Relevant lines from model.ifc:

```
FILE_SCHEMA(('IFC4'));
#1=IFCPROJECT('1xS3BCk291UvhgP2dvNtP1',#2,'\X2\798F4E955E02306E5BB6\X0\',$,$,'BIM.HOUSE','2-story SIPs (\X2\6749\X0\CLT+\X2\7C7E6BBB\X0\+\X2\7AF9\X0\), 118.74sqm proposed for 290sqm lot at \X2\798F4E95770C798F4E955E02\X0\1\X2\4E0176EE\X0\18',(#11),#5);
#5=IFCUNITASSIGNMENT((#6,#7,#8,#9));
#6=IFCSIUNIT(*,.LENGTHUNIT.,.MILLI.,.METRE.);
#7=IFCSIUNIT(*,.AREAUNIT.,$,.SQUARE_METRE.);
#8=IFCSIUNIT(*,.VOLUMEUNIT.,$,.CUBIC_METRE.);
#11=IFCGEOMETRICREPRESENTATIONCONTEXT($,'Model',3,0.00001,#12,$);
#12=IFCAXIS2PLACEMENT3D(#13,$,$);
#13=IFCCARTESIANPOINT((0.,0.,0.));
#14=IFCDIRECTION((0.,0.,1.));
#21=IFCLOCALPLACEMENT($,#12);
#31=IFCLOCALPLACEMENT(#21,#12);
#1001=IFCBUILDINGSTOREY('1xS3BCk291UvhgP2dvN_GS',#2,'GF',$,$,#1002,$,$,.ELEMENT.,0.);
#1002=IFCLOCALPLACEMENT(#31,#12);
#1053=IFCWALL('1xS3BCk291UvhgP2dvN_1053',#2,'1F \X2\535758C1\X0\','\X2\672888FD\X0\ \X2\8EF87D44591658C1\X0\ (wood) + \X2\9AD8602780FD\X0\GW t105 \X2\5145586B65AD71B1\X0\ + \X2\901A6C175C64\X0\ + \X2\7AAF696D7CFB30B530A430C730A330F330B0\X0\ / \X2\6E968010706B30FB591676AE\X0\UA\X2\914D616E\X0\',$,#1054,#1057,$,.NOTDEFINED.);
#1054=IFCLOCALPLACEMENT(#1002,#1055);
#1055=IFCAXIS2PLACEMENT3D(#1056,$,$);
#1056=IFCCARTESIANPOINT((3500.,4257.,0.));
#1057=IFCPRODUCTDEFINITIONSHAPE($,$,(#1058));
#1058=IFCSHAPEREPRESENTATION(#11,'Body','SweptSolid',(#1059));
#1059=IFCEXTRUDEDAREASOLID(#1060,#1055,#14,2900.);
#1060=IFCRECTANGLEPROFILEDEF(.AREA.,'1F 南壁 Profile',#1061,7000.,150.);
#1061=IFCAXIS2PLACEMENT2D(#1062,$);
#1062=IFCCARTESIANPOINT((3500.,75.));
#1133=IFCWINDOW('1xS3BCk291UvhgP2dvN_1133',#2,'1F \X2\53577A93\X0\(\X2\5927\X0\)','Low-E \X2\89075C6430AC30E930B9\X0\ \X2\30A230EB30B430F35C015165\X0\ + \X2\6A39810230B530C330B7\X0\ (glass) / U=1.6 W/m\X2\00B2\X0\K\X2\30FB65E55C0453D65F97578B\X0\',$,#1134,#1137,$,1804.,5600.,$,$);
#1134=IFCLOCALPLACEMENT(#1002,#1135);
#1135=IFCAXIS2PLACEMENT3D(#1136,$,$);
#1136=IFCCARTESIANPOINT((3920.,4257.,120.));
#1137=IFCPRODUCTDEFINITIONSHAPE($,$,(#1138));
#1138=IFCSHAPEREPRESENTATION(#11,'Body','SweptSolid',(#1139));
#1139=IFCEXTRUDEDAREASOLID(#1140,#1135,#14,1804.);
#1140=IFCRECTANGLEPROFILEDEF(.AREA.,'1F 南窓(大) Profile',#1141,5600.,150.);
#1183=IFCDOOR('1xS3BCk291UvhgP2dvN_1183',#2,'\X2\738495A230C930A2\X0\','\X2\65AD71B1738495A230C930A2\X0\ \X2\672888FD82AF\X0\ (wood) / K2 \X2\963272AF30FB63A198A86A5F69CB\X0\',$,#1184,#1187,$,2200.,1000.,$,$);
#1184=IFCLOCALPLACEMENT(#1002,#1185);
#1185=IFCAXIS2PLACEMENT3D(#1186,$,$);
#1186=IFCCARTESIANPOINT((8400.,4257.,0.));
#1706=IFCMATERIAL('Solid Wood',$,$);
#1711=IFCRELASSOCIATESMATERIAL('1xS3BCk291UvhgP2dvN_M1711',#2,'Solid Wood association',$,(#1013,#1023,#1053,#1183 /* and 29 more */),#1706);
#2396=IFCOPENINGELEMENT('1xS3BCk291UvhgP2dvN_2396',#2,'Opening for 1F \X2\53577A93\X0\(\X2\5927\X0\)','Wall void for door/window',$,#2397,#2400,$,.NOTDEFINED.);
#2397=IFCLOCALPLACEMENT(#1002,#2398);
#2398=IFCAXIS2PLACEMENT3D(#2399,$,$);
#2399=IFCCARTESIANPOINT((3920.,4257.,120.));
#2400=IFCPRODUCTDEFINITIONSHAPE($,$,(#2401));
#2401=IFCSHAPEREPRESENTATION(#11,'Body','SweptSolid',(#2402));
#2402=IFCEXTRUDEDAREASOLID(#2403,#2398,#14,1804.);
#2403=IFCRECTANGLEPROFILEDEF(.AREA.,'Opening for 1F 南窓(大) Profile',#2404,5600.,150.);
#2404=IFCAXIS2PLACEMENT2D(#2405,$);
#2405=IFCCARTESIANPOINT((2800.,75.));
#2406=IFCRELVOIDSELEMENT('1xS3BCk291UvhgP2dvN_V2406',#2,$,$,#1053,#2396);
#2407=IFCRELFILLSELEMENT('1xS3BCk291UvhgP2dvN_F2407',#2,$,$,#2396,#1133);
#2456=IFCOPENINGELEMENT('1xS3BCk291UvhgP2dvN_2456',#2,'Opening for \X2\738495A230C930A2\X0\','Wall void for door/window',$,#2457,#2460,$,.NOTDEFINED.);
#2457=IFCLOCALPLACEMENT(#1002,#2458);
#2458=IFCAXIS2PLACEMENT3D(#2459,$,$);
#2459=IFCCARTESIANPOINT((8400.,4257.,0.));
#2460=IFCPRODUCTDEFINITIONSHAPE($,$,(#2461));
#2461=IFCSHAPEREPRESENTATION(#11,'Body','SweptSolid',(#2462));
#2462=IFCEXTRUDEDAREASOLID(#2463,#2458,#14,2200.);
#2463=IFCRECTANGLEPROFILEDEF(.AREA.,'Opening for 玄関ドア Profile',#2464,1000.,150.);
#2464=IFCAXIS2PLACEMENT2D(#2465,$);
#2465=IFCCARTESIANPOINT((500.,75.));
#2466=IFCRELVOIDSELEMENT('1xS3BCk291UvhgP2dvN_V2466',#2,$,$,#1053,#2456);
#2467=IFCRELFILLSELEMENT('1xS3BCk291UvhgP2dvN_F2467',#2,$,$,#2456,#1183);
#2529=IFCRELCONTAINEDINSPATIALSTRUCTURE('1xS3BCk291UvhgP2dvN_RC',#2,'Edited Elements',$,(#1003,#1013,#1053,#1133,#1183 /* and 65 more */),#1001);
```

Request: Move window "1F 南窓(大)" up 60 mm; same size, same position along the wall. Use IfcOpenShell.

```python
import numpy as np
import ifcopenshell
import ifcopenshell.api.geometry
import ifcopenshell.util.placement
import ifcopenshell.util.unit

model = ifcopenshell.open("model.ifc")
unit_scale = ifcopenshell.util.unit.calculate_unit_scale(model)

window = model.by_id(1133)
opening = window.FillsVoids[0].RelatingOpeningElement
dz = 0.06 / unit_scale

shift = np.array([0.0, 0.0, dz])
# The window is not placed relative to its opening, so move both.
for product in (opening, window):
    matrix = ifcopenshell.util.placement.get_local_placement(product.ObjectPlacement)
    matrix[:3, 3] += shift
    ifcopenshell.api.geometry.edit_object_placement(model, product=product, matrix=matrix, is_si=False)

print(f"moved by {dz * unit_scale:+.3f} m")

model.write("model-out.ifc")
```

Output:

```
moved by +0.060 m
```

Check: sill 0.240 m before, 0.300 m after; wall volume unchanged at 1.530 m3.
